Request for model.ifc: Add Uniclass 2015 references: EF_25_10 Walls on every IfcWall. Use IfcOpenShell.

First a look at what the model holds.

```python
import ifcopenshell

model = ifcopenshell.open("model.ifc")
print(model.schema)
print("classifications:", [c.Name for c in model.by_type("IfcClassification")])
for ifc_class in ("IfcDoor", "IfcRoof", "IfcStair", "IfcWall", "IfcWindow"):
    print(ifc_class, len(model.by_type(ifc_class)))
```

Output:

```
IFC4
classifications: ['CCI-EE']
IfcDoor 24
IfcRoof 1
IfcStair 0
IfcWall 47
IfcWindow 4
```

```python
import ifcopenshell
import ifcopenshell.api.classification

model = ifcopenshell.open("model.ifc")

system = ifcopenshell.api.classification.add_classification(model, classification="Uniclass 2015")

codes = {
    "IfcWall": ("EF_25_10", "Walls"),
}
for ifc_class, (code, name) in codes.items():
    products = model.by_type(ifc_class)
    ifcopenshell.api.classification.add_reference(
        model, products=products, classification=system, identification=code, name=name
    )
    print(code, len(products))

model.write("model_v2.ifc")
```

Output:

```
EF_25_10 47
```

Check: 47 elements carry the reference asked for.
